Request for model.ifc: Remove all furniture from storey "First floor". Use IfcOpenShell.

First a look at what the model holds.

```python
import ifcopenshell
import ifcopenshell.util.element

model = ifcopenshell.open("model.ifc")
print(model.schema)
storey = next(s for s in model.by_type("IfcBuildingStorey") if s.Name == "First floor")
furniture = [e for e in ifcopenshell.util.element.get_decomposition(storey) if e.is_a("IfcFurnishingElement")]
seen = {}
for e in furniture:
    element_type = ifcopenshell.util.element.get_type(e)
    name = element_type.Name if element_type not in (None, e) else None
    seen[name] = seen.get(name, 0) + 1
for name, count in sorted(seen.items(), key=str):
    print(count, "x", name)
```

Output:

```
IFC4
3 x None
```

```python
import ifcopenshell
import ifcopenshell.api.root
import ifcopenshell.util.element

model = ifcopenshell.open("model.ifc")

storey = next(s for s in model.by_type("IfcBuildingStorey") if s.Name == "First floor")
furniture = [e for e in ifcopenshell.util.element.get_decomposition(storey) if e.is_a("IfcFurnishingElement")]

for e in furniture:
    ifcopenshell.api.root.remove_product(model, product=e)
print(len(furniture), "removed")

model.write("model-out.ifc")
```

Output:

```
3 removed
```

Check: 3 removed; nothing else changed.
